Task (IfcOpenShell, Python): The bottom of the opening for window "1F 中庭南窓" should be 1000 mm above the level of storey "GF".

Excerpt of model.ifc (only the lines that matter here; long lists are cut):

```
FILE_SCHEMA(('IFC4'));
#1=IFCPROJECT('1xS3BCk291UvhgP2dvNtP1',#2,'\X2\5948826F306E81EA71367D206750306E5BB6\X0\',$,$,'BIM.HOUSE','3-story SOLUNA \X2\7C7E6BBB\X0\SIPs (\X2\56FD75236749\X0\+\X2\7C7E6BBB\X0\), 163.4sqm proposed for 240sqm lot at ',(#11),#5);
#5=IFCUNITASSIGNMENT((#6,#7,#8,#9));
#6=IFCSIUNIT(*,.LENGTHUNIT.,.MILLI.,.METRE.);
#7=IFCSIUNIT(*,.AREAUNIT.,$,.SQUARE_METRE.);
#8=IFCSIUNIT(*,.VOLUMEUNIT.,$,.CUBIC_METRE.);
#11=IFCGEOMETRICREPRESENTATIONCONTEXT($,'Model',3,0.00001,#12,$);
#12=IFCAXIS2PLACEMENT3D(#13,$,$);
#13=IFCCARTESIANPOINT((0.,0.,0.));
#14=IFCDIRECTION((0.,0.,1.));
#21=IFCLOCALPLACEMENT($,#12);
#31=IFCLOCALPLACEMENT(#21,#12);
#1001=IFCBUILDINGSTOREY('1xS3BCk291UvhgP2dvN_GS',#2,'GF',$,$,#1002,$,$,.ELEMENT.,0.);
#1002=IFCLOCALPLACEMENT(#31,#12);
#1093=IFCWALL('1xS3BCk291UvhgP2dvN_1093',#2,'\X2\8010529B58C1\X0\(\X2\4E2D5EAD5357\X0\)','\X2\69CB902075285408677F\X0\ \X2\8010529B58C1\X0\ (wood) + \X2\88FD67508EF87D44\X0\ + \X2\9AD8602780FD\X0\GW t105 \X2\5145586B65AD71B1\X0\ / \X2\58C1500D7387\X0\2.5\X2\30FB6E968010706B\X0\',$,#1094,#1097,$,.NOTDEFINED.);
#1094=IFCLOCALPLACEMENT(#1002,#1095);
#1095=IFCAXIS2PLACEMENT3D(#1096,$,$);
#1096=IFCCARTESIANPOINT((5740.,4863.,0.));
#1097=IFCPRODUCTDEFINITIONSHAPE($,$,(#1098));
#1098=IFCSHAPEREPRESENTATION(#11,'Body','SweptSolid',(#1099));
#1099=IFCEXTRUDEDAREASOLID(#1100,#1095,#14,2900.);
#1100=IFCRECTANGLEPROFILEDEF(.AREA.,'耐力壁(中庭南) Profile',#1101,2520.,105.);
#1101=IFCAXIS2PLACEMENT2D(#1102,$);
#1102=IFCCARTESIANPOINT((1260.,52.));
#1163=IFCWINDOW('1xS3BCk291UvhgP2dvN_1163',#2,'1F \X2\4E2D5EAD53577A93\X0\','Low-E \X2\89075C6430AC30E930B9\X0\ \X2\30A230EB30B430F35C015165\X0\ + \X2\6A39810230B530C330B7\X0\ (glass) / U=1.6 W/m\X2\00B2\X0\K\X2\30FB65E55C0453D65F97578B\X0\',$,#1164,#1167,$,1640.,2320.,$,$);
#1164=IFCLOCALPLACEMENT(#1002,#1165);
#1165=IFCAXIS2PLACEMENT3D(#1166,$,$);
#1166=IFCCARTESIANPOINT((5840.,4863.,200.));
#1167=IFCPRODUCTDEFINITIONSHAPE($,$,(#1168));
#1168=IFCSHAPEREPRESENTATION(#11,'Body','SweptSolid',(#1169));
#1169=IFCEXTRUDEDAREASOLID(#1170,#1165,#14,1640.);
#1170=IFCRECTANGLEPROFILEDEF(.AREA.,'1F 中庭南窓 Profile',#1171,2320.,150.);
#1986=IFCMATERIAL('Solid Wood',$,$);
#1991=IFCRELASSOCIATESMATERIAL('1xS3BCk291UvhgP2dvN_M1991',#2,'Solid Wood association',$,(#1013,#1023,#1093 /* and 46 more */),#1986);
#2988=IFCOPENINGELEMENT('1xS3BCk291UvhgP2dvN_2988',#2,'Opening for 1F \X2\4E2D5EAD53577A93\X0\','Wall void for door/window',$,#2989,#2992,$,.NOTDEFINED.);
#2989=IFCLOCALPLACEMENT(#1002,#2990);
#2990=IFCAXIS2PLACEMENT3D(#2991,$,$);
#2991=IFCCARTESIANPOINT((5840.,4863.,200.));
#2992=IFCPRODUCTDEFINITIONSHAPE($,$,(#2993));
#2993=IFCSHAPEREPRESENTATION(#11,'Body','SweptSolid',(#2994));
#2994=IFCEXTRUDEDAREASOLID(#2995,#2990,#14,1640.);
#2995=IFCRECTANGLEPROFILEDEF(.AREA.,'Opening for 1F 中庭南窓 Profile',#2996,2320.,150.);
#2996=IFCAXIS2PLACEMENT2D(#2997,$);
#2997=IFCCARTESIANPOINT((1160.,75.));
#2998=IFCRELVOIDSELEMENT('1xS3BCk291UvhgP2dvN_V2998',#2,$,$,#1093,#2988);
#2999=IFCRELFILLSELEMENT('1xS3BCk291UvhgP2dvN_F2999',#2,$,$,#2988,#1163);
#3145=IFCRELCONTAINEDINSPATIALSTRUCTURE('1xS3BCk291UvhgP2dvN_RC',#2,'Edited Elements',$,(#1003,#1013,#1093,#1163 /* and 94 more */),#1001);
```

```python
import numpy as np
import ifcopenshell
import ifcopenshell.api.geometry
import ifcopenshell.geom
import ifcopenshell.util.element
import ifcopenshell.util.placement
import ifcopenshell.util.shape
import ifcopenshell.util.unit

model = ifcopenshell.open("model.ifc")
unit_scale = ifcopenshell.util.unit.calculate_unit_scale(model)

window = model.by_id(1163)
opening = window.FillsVoids[0].RelatingOpeningElement
storey = ifcopenshell.util.element.get_container(window, ifc_class="IfcBuildingStorey")
level = ifcopenshell.util.placement.get_local_placement(storey.ObjectPlacement)[2, 3]

# The opening's origin need not be at the sill, so measure its lowest point.
shape = ifcopenshell.geom.create_shape(ifcopenshell.geom.settings(), opening)
bottom = ifcopenshell.util.shape.get_shape_bottom_elevation(shape, shape.geometry) / unit_scale
dz = level + 1000.0 - bottom

shift = np.array([0.0, 0.0, dz])
# The window is not placed relative to its opening, so move both.
for product in (opening, window):
    matrix = ifcopenshell.util.placement.get_local_placement(product.ObjectPlacement)
    matrix[:3, 3] += shift
    ifcopenshell.api.geometry.edit_object_placement(model, product=product, matrix=matrix, is_si=False)

print(f"moved by {dz * unit_scale:+.3f} m")

model.write("model_v2.ifc")
```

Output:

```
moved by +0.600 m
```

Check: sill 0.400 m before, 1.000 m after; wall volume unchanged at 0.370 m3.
